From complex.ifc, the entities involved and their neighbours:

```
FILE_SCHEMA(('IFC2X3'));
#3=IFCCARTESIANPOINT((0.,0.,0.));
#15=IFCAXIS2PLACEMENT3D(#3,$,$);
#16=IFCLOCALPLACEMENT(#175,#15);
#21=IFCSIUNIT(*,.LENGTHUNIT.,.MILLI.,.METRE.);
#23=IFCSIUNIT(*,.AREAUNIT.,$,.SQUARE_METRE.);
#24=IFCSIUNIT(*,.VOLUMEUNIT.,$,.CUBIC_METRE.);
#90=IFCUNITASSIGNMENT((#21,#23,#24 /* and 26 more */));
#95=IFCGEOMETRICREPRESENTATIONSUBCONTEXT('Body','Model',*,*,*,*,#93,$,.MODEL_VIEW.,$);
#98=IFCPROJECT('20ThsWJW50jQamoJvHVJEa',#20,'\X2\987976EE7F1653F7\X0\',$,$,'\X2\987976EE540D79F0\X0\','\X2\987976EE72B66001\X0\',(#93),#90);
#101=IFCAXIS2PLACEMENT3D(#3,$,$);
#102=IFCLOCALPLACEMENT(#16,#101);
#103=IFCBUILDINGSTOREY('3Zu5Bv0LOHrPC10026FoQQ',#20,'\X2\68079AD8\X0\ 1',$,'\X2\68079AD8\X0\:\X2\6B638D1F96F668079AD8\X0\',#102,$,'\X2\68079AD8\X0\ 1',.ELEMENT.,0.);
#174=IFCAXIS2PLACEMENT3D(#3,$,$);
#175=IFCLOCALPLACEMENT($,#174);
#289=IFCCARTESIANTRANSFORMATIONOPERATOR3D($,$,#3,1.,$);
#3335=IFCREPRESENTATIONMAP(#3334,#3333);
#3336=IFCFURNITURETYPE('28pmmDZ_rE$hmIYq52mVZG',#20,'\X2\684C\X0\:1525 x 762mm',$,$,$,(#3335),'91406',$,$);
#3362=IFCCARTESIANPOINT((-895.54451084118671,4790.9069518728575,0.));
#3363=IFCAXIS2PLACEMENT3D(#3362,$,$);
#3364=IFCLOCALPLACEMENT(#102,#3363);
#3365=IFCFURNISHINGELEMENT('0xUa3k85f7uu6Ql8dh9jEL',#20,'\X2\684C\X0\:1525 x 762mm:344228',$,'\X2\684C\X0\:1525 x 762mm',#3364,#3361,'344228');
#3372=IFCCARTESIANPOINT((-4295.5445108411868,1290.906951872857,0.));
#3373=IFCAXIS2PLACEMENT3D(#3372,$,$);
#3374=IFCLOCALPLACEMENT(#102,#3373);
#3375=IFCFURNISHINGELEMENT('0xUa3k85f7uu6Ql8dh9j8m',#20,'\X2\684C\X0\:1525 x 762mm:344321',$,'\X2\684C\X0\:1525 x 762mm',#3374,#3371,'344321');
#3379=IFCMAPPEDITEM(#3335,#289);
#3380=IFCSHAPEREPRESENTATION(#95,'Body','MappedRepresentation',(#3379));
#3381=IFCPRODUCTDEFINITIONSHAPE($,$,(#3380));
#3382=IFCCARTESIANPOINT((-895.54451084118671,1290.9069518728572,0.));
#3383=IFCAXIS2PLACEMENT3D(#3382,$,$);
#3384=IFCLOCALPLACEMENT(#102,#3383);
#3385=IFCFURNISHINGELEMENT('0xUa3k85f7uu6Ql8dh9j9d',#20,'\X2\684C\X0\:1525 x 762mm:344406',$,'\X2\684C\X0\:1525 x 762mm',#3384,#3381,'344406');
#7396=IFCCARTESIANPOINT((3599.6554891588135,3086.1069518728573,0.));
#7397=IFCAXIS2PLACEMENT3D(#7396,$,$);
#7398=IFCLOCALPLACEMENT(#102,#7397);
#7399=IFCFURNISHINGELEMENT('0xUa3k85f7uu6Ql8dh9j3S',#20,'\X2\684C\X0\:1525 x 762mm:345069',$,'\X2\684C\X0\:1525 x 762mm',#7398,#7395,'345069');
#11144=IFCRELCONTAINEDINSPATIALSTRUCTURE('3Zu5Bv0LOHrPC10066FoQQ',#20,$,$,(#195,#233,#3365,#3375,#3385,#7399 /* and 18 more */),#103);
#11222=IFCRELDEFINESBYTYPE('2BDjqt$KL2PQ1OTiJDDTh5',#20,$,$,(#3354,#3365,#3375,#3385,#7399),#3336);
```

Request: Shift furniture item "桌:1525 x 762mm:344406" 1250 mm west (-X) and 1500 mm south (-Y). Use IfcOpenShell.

```python
import ifcopenshell
import ifcopenshell.api.geometry
import ifcopenshell.util.placement
import ifcopenshell.util.unit

model = ifcopenshell.open("complex.ifc")
unit_scale = ifcopenshell.util.unit.calculate_unit_scale(model)

item = model.by_id(3385)
matrix = ifcopenshell.util.placement.get_local_placement(item.ObjectPlacement)
matrix[0, 3] -= 1.25 / unit_scale
matrix[1, 3] -= 1.5 / unit_scale
ifcopenshell.api.geometry.edit_object_placement(model, product=item, matrix=matrix, is_si=False)

print(ifcopenshell.util.placement.get_local_placement(item.ObjectPlacement).round(3) + 0.0)

model.write("complex_edited.ifc")
```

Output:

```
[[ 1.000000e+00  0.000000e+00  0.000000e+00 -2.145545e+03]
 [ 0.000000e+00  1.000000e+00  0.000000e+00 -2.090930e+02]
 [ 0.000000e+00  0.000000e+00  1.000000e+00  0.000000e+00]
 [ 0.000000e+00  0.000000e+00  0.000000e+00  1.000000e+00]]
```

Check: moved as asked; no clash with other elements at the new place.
